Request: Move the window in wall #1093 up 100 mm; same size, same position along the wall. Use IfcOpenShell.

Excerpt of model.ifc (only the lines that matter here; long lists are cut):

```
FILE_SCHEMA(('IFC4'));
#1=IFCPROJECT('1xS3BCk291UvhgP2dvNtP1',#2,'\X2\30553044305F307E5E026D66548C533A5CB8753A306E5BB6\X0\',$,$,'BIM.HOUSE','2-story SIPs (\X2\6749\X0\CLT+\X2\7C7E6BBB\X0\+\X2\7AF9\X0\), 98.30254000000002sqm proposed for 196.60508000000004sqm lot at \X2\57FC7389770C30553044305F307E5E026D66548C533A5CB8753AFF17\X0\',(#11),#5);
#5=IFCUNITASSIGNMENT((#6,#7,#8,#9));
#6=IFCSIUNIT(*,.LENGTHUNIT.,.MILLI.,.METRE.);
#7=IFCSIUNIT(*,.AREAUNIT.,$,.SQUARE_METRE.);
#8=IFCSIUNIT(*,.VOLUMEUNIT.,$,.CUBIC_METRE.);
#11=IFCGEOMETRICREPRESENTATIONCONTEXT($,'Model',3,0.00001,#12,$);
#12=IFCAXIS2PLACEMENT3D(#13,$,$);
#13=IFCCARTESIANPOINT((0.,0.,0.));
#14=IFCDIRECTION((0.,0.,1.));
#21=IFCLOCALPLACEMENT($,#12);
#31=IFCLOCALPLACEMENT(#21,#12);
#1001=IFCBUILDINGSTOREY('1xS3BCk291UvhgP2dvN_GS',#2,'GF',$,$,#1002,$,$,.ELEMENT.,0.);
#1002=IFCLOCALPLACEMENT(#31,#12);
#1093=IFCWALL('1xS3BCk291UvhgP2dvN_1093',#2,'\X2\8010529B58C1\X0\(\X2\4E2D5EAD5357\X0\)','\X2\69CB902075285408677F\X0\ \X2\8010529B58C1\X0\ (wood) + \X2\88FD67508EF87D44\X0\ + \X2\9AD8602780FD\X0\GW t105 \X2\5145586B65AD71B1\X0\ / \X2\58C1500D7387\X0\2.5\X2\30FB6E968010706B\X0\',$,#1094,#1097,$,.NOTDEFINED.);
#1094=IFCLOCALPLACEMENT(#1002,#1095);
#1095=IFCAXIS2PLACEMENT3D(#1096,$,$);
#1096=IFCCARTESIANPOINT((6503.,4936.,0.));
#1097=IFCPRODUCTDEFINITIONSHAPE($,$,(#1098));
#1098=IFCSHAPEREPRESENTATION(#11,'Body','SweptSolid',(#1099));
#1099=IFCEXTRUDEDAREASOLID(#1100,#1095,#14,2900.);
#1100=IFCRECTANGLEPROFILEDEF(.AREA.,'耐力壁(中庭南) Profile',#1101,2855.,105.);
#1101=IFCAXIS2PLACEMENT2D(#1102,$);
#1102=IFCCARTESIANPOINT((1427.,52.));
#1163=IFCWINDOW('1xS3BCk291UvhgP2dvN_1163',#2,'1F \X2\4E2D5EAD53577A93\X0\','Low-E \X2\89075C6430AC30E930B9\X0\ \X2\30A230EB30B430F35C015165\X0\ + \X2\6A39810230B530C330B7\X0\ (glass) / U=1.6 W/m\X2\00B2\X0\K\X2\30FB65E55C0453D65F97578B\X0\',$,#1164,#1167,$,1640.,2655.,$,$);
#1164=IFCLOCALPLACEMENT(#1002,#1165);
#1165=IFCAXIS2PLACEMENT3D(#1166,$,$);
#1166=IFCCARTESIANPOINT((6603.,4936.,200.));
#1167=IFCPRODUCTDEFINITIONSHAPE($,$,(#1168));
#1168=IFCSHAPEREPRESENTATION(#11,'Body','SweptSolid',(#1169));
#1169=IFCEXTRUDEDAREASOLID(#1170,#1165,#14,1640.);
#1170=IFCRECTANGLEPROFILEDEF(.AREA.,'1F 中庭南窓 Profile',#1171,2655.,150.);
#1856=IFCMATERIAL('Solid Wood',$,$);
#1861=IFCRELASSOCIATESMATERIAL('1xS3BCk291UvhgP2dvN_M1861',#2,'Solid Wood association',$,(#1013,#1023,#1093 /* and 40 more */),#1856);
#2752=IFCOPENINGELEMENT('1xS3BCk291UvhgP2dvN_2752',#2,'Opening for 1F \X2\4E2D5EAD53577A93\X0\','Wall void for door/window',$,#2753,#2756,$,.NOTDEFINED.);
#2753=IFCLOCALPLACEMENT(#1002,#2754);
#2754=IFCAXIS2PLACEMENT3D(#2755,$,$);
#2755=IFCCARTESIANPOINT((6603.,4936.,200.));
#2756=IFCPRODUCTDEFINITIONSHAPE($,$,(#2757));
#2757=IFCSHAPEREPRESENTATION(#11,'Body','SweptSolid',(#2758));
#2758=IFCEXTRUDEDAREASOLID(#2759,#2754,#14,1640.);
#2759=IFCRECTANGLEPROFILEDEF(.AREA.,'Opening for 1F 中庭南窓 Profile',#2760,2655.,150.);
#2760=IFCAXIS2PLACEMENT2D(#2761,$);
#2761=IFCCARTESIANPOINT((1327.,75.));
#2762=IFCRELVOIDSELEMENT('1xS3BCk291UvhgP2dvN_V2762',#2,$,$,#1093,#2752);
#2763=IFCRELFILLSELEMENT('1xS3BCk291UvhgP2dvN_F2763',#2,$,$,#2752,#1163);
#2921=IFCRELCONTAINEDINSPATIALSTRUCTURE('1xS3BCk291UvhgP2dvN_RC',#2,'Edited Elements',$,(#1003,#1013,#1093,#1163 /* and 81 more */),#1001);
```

```python
import numpy as np
import ifcopenshell
import ifcopenshell.api.geometry
import ifcopenshell.util.placement
import ifcopenshell.util.unit

model = ifcopenshell.open("model.ifc")
unit_scale = ifcopenshell.util.unit.calculate_unit_scale(model)

window = model.by_guid("1xS3BCk291UvhgP2dvN_1163")
opening = window.FillsVoids[0].RelatingOpeningElement
dz = 0.1 / unit_scale

shift = np.array([0.0, 0.0, dz])
# The window is not placed relative to its opening, so move both.
for product in (opening, window):
    matrix = ifcopenshell.util.placement.get_local_placement(product.ObjectPlacement)
    matrix[:3, 3] += shift
    ifcopenshell.api.geometry.edit_object_placement(model, product=product, matrix=matrix, is_si=False)

print(f"moved by {dz * unit_scale:+.3f} m")

model.write("model_v2.ifc")
```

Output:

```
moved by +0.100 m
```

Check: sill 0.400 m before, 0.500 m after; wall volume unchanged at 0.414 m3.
